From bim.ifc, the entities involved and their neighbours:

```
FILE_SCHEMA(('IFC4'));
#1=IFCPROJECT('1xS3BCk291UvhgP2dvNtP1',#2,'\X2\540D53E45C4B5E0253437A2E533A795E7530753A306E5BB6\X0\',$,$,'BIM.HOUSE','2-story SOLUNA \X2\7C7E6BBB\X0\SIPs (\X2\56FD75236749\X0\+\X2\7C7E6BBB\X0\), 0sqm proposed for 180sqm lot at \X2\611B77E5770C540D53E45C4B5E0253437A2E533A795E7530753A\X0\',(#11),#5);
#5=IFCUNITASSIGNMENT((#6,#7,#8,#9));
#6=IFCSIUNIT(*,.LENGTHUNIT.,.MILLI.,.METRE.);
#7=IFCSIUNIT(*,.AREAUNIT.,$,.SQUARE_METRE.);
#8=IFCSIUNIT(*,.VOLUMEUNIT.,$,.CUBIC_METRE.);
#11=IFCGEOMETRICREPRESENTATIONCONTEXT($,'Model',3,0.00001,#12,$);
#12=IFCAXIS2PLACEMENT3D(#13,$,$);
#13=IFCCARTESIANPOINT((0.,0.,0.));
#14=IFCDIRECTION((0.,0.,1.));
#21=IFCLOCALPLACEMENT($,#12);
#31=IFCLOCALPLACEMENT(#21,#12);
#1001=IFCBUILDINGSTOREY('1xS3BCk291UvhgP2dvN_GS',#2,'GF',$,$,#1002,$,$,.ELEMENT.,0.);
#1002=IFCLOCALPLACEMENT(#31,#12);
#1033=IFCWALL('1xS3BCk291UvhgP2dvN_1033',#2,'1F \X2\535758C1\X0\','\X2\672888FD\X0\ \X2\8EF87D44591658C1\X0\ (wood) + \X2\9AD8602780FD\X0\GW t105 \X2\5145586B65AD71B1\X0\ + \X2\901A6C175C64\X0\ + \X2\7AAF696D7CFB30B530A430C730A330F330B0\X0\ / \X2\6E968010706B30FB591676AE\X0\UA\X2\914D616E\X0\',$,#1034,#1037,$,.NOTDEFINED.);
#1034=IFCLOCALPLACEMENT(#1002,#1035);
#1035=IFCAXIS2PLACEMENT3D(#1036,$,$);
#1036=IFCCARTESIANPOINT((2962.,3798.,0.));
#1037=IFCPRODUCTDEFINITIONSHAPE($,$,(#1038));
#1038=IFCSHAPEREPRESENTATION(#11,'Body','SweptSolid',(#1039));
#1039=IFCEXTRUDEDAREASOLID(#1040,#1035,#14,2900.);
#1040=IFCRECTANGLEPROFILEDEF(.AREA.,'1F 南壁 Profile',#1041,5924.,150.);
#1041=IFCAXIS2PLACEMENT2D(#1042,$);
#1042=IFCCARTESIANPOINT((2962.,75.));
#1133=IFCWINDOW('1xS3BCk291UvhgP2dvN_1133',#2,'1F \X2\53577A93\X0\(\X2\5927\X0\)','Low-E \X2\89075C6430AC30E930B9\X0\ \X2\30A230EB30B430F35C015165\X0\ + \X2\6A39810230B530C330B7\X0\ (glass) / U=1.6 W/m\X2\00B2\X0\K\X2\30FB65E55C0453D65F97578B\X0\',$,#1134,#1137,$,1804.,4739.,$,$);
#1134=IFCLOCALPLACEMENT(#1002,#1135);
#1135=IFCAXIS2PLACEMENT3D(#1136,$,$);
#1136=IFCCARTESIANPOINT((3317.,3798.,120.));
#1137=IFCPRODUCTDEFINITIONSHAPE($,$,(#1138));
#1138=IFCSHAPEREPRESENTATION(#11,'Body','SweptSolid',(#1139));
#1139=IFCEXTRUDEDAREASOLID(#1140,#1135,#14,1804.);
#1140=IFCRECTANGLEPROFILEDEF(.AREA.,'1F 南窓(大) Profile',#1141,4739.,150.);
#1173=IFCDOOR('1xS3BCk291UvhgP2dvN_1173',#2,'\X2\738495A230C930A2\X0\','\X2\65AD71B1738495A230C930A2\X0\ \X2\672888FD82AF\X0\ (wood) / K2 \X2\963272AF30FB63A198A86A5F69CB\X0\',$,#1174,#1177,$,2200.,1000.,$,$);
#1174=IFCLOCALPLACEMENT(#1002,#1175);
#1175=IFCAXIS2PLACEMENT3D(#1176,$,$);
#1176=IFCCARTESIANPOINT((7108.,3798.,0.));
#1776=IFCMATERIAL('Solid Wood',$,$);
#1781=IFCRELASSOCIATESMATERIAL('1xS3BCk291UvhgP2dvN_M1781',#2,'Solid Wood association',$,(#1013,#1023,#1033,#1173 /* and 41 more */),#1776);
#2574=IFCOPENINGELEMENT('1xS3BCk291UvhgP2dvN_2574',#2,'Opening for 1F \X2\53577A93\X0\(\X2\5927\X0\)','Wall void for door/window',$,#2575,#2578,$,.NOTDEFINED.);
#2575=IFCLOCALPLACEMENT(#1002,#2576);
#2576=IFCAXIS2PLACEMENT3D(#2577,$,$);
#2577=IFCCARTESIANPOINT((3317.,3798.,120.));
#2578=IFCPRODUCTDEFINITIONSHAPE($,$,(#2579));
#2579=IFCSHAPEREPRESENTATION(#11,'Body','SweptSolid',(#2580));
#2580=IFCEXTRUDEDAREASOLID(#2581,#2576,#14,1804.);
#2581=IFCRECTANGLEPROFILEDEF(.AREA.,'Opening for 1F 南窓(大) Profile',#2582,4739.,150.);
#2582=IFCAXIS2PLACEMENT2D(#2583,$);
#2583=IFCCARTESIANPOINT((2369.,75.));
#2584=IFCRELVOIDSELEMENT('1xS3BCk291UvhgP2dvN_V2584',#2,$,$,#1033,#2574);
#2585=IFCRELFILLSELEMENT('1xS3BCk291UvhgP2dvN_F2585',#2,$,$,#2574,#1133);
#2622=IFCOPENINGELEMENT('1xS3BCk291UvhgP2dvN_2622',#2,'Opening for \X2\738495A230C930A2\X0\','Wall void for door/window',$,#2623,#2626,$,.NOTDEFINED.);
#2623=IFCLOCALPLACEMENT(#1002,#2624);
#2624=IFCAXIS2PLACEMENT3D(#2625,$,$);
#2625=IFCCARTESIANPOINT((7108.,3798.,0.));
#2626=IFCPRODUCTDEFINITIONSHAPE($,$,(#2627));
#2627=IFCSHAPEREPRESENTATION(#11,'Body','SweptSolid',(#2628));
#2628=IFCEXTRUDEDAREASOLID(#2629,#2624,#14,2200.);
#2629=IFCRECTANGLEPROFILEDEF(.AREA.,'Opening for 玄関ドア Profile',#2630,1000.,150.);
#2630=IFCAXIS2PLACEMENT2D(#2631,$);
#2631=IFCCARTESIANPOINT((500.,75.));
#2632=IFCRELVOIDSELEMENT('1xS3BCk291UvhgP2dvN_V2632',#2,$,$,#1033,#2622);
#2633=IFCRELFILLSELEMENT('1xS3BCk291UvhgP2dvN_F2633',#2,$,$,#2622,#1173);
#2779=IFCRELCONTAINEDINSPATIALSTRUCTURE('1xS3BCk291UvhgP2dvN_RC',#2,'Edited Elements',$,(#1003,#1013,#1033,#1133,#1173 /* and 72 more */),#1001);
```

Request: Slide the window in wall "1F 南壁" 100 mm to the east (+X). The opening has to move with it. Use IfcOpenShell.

```python
import ifcopenshell
import ifcopenshell.api.geometry
import ifcopenshell.util.placement
import ifcopenshell.util.unit

model = ifcopenshell.open("bim.ifc")
unit_scale = ifcopenshell.util.unit.calculate_unit_scale(model)

window = model.by_guid("1xS3BCk291UvhgP2dvN_1133")
opening = window.FillsVoids[0].RelatingOpeningElement
wall = opening.VoidsElements[0].RelatingBuildingElement

wall_matrix = ifcopenshell.util.placement.get_local_placement(wall.ObjectPlacement)
shift = wall_matrix[:3, 0] * 0.1 / unit_scale
before = ifcopenshell.util.placement.get_local_placement(window.ObjectPlacement)[:3, 3].copy()

# The window is not placed relative to its opening, so move both.
for product in (opening, window):
    matrix = ifcopenshell.util.placement.get_local_placement(product.ObjectPlacement)
    matrix[:3, 3] += shift
    ifcopenshell.api.geometry.edit_object_placement(model, product=product, matrix=matrix, is_si=False)

after = ifcopenshell.util.placement.get_local_placement(window.ObjectPlacement)[:3, 3]
print("window moved by", (after - before).round(3) + 0.0)

model.write("bim_edited.ifc")
```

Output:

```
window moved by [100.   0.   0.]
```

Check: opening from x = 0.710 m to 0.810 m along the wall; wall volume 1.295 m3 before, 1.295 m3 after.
